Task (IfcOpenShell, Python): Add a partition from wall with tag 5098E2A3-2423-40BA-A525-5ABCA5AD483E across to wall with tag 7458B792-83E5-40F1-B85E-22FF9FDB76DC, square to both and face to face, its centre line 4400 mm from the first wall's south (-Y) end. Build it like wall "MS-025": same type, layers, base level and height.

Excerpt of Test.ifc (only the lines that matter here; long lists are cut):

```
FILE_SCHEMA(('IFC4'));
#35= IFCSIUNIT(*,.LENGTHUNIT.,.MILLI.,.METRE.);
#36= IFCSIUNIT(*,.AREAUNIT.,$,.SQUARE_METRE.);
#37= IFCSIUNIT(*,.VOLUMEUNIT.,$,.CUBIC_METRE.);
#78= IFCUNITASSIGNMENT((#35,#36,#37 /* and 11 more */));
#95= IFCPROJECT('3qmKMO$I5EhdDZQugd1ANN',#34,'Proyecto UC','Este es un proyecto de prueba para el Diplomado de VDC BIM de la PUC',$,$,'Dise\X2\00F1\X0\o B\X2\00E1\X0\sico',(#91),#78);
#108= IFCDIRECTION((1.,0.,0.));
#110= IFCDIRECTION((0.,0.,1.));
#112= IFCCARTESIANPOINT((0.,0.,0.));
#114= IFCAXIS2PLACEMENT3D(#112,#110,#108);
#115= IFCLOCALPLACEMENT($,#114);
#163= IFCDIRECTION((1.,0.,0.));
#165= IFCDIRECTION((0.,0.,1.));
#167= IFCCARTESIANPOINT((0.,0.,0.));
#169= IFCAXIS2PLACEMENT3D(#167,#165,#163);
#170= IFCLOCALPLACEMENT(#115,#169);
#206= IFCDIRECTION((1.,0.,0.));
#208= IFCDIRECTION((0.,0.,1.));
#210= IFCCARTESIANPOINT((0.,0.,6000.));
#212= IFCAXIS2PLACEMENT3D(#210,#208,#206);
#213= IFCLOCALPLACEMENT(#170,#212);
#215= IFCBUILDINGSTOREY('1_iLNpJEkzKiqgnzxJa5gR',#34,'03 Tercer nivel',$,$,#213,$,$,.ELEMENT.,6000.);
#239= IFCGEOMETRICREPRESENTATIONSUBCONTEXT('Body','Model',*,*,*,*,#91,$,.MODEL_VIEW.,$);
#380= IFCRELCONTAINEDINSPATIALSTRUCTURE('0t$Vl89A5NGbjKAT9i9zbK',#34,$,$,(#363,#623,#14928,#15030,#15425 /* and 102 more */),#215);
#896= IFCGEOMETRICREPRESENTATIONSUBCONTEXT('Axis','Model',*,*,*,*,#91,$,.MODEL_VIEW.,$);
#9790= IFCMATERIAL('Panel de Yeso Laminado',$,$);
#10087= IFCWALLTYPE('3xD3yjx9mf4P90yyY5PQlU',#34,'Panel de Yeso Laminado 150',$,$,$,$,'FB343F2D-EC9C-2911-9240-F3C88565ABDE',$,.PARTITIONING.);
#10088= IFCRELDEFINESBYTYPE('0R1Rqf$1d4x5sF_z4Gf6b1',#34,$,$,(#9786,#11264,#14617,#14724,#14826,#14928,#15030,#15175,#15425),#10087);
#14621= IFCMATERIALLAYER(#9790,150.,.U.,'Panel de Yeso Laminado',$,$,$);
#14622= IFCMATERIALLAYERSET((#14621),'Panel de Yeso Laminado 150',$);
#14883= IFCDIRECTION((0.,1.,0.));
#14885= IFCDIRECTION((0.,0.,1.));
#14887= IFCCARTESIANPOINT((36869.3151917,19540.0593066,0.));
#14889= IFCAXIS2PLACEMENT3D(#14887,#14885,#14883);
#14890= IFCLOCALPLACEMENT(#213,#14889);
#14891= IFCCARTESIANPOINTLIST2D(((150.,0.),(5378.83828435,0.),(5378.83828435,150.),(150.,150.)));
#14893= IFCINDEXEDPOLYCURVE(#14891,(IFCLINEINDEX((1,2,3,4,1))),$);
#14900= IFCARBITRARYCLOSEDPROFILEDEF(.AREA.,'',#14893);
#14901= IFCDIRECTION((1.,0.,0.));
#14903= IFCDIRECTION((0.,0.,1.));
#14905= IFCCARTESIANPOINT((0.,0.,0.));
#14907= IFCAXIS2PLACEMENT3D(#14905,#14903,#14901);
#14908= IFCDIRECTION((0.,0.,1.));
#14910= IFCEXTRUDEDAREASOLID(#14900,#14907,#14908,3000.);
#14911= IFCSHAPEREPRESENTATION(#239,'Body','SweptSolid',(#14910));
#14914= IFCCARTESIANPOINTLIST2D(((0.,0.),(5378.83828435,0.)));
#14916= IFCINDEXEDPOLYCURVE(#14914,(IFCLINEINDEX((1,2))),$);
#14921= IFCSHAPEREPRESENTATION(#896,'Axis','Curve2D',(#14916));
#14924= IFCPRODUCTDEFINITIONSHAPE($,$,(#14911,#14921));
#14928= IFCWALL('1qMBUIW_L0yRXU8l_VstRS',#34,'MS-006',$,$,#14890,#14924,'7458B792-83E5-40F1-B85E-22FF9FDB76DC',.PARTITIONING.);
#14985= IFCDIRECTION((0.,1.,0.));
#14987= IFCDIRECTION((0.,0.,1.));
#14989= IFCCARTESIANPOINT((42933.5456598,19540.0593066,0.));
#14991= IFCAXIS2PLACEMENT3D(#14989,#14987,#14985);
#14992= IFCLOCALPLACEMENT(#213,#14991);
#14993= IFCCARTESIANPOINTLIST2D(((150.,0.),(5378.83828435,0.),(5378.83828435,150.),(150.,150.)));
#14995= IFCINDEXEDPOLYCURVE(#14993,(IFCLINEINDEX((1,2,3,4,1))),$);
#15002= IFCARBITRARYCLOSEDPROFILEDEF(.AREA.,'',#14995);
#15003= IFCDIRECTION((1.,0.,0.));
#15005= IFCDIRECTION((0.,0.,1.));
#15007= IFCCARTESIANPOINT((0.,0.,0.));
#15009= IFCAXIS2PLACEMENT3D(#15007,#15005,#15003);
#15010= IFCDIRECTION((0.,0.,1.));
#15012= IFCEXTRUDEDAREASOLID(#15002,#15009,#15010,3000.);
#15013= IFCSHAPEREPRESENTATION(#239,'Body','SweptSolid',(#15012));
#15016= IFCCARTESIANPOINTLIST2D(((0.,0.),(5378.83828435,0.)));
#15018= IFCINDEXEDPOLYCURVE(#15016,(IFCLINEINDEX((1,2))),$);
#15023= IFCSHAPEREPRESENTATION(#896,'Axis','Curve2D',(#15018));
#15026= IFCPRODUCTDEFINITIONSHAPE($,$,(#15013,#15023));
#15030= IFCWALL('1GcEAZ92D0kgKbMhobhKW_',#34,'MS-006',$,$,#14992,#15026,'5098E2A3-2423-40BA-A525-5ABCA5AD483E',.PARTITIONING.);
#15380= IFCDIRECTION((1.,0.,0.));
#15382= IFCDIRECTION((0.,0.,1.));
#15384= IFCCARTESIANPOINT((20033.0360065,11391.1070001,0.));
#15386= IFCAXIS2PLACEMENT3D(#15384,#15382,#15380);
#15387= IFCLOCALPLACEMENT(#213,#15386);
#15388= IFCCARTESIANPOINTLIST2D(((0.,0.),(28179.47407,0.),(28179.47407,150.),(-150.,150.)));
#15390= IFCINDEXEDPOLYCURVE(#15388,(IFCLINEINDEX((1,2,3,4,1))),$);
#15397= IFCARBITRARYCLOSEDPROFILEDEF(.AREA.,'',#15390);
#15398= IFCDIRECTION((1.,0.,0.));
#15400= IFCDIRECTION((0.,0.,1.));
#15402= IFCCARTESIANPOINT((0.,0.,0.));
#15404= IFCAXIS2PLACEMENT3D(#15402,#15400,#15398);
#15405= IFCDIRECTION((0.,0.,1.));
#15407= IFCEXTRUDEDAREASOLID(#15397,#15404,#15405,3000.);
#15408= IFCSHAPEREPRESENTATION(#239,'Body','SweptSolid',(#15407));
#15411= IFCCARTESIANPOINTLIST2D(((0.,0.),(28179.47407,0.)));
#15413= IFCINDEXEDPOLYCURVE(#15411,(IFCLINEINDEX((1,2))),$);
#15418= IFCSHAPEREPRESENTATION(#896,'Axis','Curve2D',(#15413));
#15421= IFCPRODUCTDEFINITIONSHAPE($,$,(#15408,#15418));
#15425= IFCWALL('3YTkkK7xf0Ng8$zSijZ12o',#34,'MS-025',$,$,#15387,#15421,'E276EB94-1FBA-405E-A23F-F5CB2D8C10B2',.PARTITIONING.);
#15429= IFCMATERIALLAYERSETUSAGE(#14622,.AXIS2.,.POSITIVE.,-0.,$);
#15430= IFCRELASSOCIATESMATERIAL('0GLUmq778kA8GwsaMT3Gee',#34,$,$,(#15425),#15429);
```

```python
import numpy as np
import ifcopenshell
import ifcopenshell.api.geometry
import ifcopenshell.api.material
import ifcopenshell.api.pset
import ifcopenshell.api.root
import ifcopenshell.api.spatial
import ifcopenshell.api.type
import ifcopenshell.geom
import ifcopenshell.util.element
import ifcopenshell.util.placement
import ifcopenshell.util.representation
import ifcopenshell.util.shape
import ifcopenshell.util.unit

model = ifcopenshell.open("Test.ifc")
unit_scale = ifcopenshell.util.unit.calculate_unit_scale(model)
settings = ifcopenshell.geom.settings()
settings.set("use-world-coords", True)

start_wall = model.by_guid("1GcEAZ92D0kgKbMhobhKW_")
end_wall = model.by_guid("1qMBUIW_L0yRXU8l_VstRS")
like = model.by_id(15425)
matrix = ifcopenshell.util.placement.get_local_placement(start_wall.ObjectPlacement)
matrix[:3, 3] *= unit_scale


def extent(element):
    """Bounding box in the first wall's axes, in metres."""
    shape = ifcopenshell.geom.create_shape(settings, element)
    points = (ifcopenshell.util.shape.get_vertices(shape.geometry) - matrix[:3, 3]) @ matrix[:3, :3]
    return points.min(axis=0), points.max(axis=0)


y_start = extent(start_wall)[1][1]
y_end = extent(end_wall)[0][1]
like_min, like_max = extent(like)
length, height = float(abs(y_end - y_start)), float(like_max[2] - like_min[2])
layer_set = ifcopenshell.util.element.get_material(like, should_skip_usage=True)
thickness = sum(layer.LayerThickness for layer in layer_set.MaterialLayers) * unit_scale

wall = ifcopenshell.api.root.create_entity(model, ifc_class="IfcWall", name="New partition")
storey = ifcopenshell.util.element.get_container(like)
ifcopenshell.api.spatial.assign_container(model, products=[wall], relating_structure=storey)
ifcopenshell.api.type.assign_type(
    model, related_objects=[wall], relating_type=ifcopenshell.util.element.get_type(like), should_map_representations=False
)
rel = ifcopenshell.api.material.assign_material(
    model, products=[wall], type="IfcMaterialLayerSetUsage", material=layer_set
)
rel.RelatingMaterial.OffsetFromReferenceLine = -thickness / 2 / unit_scale
pset = ifcopenshell.api.pset.add_pset(model, product=wall, name="Pset_WallCommon")
ifcopenshell.api.pset.edit_pset(model, pset=pset, properties={"IsExternal": False, "LoadBearing": False})

# The axis runs down the middle of the wall.
axis = ifcopenshell.api.geometry.add_axis_representation(
    model, context=ifcopenshell.util.representation.get_context(model, "Model", "Axis"), axis=[(0.0, 0.0), (length, 0.0)]
)
body = ifcopenshell.api.geometry.add_wall_representation(
    model,
    context=ifcopenshell.util.representation.get_context(model, "Model", "Body", "MODEL_VIEW"),
    length=length,
    height=height,
    thickness=thickness,
    offset=-thickness / 2,
)
for representation in (axis, body):
    ifcopenshell.api.geometry.assign_representation(model, product=wall, representation=representation)

placement = matrix @ ifcopenshell.util.placement.rotation(90, "Z")
placement[:, 3] = matrix @ np.array([extent(start_wall)[0][0] + 4.4, y_start, like_min[2], 1.0])
ifcopenshell.api.geometry.edit_object_placement(model, product=wall, matrix=placement)

print(f"partition {length:.3f} m long, {height:.3f} m high, {thickness:.3f} m thick")

model.write("Test-out.ifc")
```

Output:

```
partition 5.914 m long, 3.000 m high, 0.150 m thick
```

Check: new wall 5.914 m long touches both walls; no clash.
